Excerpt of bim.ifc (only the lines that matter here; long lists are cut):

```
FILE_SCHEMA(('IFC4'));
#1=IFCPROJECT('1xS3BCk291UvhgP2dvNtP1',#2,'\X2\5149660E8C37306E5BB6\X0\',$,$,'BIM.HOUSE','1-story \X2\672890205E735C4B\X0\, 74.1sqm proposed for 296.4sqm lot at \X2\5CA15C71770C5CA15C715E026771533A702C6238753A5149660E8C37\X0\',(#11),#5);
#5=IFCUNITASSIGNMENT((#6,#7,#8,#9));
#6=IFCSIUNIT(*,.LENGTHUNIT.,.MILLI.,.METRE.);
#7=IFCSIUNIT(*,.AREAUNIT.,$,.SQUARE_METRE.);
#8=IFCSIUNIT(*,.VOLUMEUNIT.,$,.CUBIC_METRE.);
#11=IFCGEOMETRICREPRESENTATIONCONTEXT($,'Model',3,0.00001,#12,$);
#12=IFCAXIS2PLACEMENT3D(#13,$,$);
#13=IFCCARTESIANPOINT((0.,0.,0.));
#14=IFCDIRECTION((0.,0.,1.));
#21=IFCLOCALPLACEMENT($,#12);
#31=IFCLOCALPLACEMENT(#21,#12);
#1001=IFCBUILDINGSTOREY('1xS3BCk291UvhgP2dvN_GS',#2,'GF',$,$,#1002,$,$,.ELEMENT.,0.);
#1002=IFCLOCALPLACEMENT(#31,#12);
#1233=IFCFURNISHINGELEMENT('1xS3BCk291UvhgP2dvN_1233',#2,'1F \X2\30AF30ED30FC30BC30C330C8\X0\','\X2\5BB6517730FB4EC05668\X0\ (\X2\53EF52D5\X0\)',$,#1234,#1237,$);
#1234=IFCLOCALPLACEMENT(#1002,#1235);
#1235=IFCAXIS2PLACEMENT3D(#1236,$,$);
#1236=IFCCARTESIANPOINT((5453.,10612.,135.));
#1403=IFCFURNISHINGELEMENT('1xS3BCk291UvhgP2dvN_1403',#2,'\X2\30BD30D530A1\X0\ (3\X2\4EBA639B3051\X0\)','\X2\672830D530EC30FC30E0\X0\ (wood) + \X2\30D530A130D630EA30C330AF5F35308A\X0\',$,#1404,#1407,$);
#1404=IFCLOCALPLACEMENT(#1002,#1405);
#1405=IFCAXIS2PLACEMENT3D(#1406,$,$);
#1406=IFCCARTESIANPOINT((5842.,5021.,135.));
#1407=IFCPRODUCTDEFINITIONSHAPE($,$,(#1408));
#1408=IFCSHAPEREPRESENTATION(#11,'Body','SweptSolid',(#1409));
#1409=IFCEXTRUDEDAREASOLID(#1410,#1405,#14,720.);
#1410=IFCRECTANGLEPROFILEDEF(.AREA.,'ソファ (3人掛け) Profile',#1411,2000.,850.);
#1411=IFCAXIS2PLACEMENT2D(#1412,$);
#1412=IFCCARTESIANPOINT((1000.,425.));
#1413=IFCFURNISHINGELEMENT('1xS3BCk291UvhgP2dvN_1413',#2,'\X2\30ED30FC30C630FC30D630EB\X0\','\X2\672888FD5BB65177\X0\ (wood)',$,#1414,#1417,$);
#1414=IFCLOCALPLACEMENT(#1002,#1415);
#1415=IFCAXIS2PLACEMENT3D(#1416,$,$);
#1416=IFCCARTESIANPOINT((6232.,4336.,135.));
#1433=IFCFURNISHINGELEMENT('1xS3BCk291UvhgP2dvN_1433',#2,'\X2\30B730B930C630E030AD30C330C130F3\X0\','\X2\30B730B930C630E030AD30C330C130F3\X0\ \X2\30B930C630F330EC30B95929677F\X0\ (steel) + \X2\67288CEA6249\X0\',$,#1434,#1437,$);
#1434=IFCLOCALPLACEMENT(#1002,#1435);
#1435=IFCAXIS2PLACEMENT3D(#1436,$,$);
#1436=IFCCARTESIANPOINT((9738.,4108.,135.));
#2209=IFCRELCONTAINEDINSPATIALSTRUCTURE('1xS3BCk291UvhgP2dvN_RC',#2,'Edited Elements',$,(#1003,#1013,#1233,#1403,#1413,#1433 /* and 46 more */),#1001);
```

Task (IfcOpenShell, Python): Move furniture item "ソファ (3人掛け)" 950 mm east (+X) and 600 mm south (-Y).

```python
import ifcopenshell
import ifcopenshell.api.geometry
import ifcopenshell.util.placement
import ifcopenshell.util.unit

model = ifcopenshell.open("bim.ifc")
unit_scale = ifcopenshell.util.unit.calculate_unit_scale(model)

item = model.by_guid("1xS3BCk291UvhgP2dvN_1403")
matrix = ifcopenshell.util.placement.get_local_placement(item.ObjectPlacement)
matrix[0, 3] += 0.95 / unit_scale
matrix[1, 3] -= 0.6 / unit_scale
ifcopenshell.api.geometry.edit_object_placement(model, product=item, matrix=matrix, is_si=False)

print(ifcopenshell.util.placement.get_local_placement(item.ObjectPlacement).round(3) + 0.0)

model.write("bim_v2.ifc")
```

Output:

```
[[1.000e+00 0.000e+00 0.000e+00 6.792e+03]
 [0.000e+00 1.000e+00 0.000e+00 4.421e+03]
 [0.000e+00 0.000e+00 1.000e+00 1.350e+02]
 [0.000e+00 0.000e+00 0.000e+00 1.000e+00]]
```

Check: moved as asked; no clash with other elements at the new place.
